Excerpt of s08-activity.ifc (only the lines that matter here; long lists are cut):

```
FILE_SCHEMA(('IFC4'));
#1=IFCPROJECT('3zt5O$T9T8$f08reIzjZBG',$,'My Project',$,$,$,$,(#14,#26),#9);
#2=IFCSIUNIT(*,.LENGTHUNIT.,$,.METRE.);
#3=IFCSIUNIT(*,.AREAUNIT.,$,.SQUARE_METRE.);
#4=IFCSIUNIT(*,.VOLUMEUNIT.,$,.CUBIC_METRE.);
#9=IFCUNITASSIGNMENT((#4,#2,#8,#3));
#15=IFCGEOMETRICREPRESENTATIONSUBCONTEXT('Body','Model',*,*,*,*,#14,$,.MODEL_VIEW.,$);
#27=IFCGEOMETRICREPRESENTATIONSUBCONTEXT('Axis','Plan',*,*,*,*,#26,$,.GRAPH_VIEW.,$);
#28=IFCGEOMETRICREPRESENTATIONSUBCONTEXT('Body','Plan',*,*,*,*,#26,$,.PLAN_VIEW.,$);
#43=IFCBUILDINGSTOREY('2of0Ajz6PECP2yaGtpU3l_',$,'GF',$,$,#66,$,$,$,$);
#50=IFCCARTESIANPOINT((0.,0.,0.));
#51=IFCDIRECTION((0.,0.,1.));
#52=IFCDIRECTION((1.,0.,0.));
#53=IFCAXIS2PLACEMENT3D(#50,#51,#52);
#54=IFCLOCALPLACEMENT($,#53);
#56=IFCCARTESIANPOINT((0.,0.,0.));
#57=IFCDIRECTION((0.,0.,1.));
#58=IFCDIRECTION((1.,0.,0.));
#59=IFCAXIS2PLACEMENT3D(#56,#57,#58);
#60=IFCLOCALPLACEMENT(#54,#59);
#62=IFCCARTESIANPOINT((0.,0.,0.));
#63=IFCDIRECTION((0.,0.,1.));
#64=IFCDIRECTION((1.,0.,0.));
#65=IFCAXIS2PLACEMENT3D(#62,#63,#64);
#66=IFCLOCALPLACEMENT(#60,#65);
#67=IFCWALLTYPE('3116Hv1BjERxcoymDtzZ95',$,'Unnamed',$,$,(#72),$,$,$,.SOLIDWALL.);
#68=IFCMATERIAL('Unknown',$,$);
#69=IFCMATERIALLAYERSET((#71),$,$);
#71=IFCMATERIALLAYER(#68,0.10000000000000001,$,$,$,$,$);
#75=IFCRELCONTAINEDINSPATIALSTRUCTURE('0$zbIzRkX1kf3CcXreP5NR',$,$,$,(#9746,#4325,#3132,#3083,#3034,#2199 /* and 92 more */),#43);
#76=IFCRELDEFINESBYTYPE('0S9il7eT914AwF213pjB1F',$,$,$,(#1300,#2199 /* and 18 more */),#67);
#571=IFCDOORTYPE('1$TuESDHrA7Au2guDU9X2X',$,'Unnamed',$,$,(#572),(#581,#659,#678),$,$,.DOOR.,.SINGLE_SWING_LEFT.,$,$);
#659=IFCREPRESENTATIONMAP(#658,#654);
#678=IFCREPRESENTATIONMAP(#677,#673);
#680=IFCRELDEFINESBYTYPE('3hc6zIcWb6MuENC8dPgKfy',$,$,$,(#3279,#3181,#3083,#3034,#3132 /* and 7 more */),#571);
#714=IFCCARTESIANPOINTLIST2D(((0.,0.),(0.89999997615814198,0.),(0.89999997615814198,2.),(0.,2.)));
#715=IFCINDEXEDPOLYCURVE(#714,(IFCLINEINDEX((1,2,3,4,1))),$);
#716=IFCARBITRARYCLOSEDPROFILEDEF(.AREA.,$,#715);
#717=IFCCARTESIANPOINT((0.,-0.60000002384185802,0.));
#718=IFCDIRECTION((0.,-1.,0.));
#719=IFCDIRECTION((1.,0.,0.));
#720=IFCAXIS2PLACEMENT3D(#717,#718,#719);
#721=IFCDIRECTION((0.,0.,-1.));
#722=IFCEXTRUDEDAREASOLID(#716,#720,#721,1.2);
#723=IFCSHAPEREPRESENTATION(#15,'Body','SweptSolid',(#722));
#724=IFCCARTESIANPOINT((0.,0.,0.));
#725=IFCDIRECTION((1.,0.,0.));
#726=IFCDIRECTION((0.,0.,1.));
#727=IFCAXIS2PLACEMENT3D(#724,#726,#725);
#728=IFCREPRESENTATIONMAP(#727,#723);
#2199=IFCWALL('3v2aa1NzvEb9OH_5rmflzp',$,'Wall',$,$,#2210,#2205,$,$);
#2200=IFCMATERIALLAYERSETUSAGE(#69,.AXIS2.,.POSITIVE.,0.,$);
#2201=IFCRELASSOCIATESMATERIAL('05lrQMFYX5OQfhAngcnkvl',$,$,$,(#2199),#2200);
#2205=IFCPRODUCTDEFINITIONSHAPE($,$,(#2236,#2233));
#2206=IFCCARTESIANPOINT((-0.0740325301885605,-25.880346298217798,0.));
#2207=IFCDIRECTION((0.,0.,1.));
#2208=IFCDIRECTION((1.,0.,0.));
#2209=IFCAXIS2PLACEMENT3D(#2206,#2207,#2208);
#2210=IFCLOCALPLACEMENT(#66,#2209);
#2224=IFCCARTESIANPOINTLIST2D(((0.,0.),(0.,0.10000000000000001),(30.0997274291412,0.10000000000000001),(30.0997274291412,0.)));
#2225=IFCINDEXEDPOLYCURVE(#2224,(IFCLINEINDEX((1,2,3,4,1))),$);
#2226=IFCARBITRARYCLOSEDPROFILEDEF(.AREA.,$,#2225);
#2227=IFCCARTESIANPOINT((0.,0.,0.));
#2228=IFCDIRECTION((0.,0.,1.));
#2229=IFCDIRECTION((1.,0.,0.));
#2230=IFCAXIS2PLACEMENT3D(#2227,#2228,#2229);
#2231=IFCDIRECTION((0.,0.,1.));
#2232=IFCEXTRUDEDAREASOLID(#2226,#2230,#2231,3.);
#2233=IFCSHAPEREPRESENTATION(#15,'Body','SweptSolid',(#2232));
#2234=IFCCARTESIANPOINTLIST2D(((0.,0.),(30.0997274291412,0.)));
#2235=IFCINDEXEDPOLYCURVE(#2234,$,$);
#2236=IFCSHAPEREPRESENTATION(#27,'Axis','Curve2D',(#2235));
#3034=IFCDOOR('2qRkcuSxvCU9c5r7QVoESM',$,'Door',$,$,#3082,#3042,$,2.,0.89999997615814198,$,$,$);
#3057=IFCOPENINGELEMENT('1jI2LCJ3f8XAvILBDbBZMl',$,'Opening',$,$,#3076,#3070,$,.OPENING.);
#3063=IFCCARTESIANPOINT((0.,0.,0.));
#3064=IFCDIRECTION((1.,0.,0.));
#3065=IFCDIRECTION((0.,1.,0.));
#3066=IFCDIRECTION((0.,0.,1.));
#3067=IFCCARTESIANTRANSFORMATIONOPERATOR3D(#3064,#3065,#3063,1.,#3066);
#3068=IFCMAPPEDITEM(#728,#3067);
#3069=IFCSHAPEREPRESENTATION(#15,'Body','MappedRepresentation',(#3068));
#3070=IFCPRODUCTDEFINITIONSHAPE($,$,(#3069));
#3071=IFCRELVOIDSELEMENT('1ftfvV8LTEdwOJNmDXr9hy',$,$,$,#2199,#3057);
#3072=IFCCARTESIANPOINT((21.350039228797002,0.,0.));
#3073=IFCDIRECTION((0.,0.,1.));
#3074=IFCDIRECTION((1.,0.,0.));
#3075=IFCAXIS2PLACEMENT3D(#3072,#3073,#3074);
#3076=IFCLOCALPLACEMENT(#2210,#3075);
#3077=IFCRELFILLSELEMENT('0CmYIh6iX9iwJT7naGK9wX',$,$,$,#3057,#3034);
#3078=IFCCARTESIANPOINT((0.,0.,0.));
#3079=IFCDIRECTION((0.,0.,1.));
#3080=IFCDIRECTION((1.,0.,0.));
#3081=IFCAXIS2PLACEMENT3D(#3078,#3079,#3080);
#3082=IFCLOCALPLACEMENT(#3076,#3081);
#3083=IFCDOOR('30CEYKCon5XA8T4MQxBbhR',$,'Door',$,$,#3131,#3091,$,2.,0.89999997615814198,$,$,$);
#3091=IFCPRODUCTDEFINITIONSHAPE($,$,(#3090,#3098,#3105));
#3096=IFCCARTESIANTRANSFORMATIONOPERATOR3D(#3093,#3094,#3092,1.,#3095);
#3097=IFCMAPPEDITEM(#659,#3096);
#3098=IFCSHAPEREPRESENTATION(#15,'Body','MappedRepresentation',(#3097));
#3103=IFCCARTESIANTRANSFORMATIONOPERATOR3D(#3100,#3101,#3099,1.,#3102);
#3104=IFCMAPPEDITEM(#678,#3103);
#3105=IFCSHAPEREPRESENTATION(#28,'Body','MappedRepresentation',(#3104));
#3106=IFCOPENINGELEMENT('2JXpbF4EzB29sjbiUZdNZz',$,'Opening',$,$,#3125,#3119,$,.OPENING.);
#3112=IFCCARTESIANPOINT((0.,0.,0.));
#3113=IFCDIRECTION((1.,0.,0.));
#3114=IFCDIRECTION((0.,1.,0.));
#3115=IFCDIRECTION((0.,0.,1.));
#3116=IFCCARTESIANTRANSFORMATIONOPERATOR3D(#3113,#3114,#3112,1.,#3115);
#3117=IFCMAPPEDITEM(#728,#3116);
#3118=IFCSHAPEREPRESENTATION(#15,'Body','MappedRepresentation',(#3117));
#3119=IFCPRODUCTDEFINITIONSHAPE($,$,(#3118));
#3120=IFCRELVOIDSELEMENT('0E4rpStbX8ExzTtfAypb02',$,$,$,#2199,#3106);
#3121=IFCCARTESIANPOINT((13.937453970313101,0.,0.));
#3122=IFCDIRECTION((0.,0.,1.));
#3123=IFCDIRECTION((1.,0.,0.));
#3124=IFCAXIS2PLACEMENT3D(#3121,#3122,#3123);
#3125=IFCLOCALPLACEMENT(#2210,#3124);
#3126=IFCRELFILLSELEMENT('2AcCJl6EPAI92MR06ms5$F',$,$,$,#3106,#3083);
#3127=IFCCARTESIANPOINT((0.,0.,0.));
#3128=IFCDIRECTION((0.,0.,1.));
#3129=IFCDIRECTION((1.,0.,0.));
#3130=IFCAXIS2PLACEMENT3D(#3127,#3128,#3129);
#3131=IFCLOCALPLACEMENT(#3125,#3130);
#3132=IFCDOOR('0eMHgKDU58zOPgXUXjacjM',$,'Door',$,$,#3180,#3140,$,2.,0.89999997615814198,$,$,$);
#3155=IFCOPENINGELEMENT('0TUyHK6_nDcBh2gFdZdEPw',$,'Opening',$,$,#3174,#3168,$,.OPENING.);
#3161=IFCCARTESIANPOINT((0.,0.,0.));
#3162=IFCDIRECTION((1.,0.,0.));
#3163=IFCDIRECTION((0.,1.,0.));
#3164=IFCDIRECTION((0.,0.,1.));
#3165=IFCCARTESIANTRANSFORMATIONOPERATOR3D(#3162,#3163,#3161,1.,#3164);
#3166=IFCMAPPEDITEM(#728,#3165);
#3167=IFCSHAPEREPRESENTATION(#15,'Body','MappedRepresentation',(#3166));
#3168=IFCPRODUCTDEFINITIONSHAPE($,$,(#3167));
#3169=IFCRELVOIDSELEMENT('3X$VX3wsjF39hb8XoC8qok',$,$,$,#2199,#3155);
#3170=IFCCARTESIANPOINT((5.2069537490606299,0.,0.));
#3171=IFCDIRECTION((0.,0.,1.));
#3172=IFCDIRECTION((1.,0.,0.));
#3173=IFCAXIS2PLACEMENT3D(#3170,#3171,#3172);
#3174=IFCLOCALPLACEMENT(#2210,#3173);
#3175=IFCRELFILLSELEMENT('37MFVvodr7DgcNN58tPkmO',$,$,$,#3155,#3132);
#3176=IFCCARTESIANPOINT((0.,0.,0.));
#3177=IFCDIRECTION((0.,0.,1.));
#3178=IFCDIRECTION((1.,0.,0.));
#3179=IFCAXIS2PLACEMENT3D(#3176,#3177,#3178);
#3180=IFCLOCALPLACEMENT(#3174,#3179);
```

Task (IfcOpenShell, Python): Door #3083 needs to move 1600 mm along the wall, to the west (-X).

```python
import ifcopenshell
import ifcopenshell.api.geometry
import ifcopenshell.util.placement

model = ifcopenshell.open("s08-activity.ifc")

door = model.by_guid("30CEYKCon5XA8T4MQxBbhR")
opening = door.FillsVoids[0].RelatingOpeningElement
wall = opening.VoidsElements[0].RelatingBuildingElement

wall_matrix = ifcopenshell.util.placement.get_local_placement(wall.ObjectPlacement)
shift = wall_matrix[:3, 0] * -1.6
before = ifcopenshell.util.placement.get_local_placement(door.ObjectPlacement)[:3, 3].copy()

# The door is placed relative to its opening, so it follows when the opening moves.
matrix = ifcopenshell.util.placement.get_local_placement(opening.ObjectPlacement)
matrix[:3, 3] += shift
ifcopenshell.api.geometry.edit_object_placement(
    model, product=opening, matrix=matrix, is_si=False, should_transform_children=True
)

after = ifcopenshell.util.placement.get_local_placement(door.ObjectPlacement)[:3, 3]
print("door moved by", (after - before).round(3) + 0.0)

model.write("s08-activity_edited.ifc")
```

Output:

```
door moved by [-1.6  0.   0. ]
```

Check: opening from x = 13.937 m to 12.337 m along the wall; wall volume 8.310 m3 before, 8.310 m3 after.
